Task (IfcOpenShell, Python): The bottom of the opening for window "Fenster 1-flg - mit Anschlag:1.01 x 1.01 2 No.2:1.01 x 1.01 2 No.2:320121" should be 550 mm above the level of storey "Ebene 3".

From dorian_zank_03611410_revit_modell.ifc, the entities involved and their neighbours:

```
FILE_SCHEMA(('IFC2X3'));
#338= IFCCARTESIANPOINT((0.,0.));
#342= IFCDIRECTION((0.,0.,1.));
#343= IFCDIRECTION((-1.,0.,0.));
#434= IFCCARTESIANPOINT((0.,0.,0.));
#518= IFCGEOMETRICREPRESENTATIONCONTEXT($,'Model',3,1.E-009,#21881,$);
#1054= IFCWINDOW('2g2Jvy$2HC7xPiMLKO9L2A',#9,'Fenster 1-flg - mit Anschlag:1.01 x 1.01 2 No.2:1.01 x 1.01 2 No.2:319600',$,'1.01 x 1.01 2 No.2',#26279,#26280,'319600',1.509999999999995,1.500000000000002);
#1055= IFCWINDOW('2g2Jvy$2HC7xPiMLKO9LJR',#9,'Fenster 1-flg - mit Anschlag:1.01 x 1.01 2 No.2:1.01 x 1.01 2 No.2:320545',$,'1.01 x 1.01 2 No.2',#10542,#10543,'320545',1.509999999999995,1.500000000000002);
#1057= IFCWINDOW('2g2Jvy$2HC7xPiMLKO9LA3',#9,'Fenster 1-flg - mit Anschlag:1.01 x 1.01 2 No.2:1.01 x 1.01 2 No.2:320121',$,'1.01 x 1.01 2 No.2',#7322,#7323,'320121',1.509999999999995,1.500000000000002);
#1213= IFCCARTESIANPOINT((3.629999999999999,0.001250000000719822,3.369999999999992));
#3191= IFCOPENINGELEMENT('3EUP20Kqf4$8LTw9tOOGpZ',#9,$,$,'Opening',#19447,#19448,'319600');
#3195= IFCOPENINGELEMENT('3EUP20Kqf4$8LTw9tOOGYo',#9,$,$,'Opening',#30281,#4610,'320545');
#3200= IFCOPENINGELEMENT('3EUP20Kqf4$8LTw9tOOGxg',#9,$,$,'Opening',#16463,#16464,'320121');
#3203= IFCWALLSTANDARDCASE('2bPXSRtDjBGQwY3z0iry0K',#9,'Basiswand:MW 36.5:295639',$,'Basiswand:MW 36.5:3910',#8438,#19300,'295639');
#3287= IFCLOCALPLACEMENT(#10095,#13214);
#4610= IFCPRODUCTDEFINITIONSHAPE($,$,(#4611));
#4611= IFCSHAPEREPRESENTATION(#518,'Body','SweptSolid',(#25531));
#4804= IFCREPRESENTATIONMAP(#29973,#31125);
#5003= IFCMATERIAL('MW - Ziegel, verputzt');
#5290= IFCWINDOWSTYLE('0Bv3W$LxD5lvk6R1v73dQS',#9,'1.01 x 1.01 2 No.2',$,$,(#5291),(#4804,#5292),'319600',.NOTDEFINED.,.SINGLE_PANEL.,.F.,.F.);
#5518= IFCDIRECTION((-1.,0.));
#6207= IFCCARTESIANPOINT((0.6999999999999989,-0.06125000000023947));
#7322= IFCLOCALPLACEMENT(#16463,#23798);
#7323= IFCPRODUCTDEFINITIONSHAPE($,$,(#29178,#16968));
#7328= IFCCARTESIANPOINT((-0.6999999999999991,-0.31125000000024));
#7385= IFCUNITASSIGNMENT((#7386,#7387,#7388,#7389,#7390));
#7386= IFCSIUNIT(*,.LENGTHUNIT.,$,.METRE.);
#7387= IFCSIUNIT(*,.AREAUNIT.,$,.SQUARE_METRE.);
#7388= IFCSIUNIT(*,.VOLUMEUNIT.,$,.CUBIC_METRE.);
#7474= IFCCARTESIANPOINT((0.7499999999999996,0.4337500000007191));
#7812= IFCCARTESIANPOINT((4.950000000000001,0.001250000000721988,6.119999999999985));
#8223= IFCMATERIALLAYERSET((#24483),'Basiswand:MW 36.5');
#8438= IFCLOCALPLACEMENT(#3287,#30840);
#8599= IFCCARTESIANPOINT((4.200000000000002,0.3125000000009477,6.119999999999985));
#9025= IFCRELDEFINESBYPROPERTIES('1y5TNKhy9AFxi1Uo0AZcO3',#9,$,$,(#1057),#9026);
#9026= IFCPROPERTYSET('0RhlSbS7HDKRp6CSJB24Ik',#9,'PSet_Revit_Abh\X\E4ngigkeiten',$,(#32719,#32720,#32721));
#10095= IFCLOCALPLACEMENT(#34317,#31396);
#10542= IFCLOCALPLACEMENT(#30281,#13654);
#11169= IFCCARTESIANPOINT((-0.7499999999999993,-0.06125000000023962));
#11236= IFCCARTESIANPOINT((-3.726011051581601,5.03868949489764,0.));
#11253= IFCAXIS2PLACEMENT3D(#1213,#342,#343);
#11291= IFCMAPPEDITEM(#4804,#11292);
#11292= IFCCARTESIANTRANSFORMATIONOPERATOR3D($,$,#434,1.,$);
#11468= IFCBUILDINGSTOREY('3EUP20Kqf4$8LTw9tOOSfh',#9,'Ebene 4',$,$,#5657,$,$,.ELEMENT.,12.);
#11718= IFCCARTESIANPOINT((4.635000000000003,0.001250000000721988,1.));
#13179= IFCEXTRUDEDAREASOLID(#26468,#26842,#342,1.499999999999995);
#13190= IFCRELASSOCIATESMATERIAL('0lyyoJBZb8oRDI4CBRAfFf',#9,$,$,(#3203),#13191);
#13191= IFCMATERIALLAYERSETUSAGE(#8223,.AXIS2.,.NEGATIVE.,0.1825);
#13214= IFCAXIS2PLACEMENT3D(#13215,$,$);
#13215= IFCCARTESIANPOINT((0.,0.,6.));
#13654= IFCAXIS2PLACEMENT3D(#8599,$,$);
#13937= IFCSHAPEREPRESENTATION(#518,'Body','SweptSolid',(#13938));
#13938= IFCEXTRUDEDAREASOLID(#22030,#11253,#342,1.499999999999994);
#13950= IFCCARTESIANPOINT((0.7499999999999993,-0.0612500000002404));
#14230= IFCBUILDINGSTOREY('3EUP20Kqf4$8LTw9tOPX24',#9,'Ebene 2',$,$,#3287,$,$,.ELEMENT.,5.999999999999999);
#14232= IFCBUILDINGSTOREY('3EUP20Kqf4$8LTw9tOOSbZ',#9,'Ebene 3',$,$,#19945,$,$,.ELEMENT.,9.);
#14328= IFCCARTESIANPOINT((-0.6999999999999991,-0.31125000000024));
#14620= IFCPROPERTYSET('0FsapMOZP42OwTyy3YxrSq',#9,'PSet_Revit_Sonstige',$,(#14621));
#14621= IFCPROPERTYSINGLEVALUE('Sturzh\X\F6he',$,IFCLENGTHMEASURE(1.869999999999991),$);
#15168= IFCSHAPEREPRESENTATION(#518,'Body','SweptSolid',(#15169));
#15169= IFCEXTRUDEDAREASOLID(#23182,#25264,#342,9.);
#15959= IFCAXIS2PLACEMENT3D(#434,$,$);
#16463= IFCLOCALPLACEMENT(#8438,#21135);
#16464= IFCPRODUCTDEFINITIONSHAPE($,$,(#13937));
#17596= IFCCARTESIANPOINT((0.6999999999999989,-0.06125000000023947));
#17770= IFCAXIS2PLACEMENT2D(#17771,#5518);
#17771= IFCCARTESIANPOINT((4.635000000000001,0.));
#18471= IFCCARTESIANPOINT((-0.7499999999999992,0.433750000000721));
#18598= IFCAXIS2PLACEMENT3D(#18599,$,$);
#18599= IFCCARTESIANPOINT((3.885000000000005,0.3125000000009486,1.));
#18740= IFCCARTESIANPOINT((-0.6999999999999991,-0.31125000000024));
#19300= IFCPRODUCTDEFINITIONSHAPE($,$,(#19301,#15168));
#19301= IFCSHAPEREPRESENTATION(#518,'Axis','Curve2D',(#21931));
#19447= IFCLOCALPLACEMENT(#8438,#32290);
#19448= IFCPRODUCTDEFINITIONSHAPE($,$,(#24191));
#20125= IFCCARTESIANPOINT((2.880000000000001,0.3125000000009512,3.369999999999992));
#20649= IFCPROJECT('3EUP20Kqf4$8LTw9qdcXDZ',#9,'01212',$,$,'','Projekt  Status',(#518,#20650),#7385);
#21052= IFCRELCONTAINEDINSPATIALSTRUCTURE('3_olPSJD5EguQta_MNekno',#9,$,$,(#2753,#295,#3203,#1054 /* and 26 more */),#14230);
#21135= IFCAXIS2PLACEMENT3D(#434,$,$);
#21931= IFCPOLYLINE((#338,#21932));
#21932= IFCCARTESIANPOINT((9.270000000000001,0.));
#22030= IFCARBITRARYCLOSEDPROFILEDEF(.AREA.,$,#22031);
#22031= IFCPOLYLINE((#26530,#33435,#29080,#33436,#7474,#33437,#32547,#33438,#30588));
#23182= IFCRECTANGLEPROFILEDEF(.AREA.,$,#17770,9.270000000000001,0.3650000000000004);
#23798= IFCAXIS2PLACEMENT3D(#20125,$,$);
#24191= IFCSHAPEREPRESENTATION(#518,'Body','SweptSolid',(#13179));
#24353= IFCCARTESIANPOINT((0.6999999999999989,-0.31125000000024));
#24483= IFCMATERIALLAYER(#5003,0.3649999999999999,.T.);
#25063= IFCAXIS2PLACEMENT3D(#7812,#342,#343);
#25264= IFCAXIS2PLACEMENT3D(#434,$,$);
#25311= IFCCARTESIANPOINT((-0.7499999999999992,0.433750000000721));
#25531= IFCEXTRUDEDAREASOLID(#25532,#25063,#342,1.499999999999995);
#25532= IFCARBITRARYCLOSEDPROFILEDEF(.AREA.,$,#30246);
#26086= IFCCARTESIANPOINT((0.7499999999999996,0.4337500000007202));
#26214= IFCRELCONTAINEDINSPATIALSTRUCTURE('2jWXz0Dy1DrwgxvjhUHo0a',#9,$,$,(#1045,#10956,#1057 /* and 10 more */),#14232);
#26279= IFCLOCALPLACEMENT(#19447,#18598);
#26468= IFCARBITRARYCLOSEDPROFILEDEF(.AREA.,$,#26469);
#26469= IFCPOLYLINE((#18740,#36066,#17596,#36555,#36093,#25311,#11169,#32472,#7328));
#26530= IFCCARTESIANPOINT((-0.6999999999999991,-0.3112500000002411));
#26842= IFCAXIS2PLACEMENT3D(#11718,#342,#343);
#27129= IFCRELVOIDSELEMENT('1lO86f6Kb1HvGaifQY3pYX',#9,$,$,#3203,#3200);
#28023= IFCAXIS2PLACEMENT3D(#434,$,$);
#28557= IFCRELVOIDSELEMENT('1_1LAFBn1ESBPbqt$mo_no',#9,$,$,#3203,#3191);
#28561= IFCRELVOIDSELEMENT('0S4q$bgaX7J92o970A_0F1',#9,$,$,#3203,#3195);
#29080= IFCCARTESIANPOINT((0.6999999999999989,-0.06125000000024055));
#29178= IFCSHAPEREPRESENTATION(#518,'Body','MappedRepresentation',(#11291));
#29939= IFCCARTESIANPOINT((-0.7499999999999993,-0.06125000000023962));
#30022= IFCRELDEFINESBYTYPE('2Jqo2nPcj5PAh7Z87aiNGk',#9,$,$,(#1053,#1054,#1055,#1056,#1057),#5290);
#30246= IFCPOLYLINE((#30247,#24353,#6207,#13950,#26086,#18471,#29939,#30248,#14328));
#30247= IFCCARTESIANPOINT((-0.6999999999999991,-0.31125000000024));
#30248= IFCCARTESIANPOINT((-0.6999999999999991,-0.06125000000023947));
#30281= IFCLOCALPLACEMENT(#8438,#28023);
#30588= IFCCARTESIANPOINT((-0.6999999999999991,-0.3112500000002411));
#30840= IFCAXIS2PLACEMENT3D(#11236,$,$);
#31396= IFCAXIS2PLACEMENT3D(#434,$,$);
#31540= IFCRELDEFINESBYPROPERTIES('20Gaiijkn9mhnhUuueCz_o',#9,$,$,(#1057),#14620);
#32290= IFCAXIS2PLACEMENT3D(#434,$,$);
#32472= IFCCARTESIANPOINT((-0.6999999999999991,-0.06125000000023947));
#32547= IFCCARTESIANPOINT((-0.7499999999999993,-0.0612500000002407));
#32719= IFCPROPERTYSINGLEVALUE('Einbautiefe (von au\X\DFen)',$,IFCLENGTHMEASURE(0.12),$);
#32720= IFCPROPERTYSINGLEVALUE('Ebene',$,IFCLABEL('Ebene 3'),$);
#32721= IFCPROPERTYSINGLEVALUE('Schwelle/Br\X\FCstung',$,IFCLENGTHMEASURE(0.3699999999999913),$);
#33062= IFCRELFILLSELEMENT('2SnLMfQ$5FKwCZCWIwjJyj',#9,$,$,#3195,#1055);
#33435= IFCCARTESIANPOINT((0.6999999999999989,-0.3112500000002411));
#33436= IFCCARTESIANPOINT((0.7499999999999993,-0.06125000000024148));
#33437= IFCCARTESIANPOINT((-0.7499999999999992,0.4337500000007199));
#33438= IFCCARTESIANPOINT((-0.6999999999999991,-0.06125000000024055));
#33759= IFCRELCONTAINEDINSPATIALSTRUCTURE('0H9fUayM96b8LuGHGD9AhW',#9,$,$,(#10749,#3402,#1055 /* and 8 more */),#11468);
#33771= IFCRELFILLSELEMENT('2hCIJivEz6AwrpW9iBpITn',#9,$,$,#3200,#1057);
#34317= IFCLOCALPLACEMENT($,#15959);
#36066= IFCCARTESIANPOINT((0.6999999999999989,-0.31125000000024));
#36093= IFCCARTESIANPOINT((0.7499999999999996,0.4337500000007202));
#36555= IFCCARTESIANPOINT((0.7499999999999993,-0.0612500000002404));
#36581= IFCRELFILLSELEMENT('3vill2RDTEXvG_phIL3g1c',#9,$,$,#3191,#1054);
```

```python
import numpy as np
import ifcopenshell
import ifcopenshell.api.geometry
import ifcopenshell.api.pset
import ifcopenshell.geom
import ifcopenshell.util.element
import ifcopenshell.util.placement
import ifcopenshell.util.shape
import ifcopenshell.util.unit

model = ifcopenshell.open("dorian_zank_03611410_revit_modell.ifc")
unit_scale = ifcopenshell.util.unit.calculate_unit_scale(model)

window = model.by_guid("2g2Jvy$2HC7xPiMLKO9LA3")
opening = window.FillsVoids[0].RelatingOpeningElement
storey = ifcopenshell.util.element.get_container(window, ifc_class="IfcBuildingStorey")
level = ifcopenshell.util.placement.get_local_placement(storey.ObjectPlacement)[2, 3]

# The opening's origin need not be at the sill, so measure its lowest point.
shape = ifcopenshell.geom.create_shape(ifcopenshell.geom.settings(), opening)
bottom = ifcopenshell.util.shape.get_shape_bottom_elevation(shape, shape.geometry) / unit_scale
dz = level + 0.55 - bottom

shift = np.array([0.0, 0.0, dz])
# The window is placed relative to its opening, so it follows when the opening moves.
matrix = ifcopenshell.util.placement.get_local_placement(opening.ObjectPlacement)
matrix[:3, 3] += shift
ifcopenshell.api.geometry.edit_object_placement(
    model, product=opening, matrix=matrix, is_si=False, should_transform_children=True
)

# Keep the stored heights in step.
pset = model.by_id(ifcopenshell.util.element.get_pset(window, "PSet_Revit_Abhängigkeiten", should_inherit=False)["id"])
ifcopenshell.api.pset.edit_pset(model, pset=pset, properties={
    "Schwelle/Brüstung": model.create_entity("IfcLengthMeasure", ifcopenshell.util.element.get_pset(window, "PSet_Revit_Abhängigkeiten", "Schwelle/Brüstung") + dz),
})
pset = model.by_id(ifcopenshell.util.element.get_pset(window, "PSet_Revit_Sonstige", should_inherit=False)["id"])
ifcopenshell.api.pset.edit_pset(model, pset=pset, properties={
    "Sturzhöhe": model.create_entity("IfcLengthMeasure", ifcopenshell.util.element.get_pset(window, "PSet_Revit_Sonstige", "Sturzhöhe") + dz),
})

print(f"moved by {dz * unit_scale:+.3f} m")

model.write("dorian_zank_03611410_revit_modell_edited.ifc")
```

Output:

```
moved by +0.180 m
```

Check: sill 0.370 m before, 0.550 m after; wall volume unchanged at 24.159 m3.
